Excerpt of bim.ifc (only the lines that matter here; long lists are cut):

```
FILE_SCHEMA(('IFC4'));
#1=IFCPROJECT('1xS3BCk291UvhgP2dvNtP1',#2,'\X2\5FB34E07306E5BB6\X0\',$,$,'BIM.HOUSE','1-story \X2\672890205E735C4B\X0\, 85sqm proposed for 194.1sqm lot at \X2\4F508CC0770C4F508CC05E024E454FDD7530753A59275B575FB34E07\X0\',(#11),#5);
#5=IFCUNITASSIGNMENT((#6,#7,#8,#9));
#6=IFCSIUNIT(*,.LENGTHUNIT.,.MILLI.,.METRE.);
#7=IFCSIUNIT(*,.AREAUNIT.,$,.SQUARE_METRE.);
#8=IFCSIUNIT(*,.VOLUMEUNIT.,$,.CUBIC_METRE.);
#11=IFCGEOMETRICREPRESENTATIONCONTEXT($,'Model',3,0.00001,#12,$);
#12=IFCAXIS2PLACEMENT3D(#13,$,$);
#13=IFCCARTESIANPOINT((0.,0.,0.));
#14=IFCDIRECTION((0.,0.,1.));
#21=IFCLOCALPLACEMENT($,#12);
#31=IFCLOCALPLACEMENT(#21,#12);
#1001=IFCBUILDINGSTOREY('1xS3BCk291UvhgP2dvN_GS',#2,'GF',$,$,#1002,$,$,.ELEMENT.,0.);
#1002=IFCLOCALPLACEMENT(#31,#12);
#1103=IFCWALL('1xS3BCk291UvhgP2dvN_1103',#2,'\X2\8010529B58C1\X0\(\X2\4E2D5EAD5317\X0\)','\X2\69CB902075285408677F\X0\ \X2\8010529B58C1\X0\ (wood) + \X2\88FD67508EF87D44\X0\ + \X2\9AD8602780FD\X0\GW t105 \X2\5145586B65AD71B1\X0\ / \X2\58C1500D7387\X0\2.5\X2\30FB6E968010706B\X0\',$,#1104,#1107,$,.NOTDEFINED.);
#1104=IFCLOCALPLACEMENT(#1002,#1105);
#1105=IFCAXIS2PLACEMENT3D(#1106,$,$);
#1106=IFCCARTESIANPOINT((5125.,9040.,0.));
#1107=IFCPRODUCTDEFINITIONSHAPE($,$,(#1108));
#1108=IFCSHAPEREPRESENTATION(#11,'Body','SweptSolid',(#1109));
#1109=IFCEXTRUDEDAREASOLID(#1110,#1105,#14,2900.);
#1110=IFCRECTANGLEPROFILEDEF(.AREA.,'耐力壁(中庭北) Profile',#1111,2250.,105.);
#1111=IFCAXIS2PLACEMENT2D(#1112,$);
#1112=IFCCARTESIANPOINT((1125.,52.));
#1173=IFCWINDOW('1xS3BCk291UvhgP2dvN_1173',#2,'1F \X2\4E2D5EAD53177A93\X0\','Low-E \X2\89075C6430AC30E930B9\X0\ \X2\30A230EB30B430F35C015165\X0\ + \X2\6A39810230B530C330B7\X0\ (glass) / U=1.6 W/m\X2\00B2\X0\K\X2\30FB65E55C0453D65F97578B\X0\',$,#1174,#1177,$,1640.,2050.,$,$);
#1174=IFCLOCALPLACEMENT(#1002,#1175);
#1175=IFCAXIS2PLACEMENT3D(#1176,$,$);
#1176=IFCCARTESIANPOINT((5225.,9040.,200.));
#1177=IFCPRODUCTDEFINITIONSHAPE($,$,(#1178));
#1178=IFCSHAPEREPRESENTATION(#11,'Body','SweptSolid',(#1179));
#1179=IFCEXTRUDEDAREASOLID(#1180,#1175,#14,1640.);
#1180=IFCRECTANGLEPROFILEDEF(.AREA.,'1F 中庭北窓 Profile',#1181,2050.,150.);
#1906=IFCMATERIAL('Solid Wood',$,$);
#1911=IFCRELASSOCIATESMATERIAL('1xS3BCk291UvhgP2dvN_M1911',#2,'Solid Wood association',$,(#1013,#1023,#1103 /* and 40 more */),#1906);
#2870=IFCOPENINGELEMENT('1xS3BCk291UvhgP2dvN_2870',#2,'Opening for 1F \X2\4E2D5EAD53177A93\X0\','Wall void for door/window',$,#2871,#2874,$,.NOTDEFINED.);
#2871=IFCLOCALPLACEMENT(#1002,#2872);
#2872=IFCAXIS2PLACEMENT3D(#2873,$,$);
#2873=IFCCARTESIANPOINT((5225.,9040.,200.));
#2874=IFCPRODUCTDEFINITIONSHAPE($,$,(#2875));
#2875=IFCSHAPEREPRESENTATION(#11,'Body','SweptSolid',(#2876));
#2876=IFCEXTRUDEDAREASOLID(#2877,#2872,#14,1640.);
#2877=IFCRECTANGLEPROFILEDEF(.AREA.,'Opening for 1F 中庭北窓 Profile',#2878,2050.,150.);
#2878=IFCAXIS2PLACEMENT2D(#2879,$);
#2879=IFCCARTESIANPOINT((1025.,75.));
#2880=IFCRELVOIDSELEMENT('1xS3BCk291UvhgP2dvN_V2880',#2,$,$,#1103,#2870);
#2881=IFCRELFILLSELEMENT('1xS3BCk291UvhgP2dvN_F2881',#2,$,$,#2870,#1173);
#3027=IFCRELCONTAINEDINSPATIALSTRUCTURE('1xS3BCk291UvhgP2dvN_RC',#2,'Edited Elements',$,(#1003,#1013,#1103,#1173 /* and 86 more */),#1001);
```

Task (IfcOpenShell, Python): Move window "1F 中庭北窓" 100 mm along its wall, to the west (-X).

```python
import ifcopenshell
import ifcopenshell.api.geometry
import ifcopenshell.util.placement
import ifcopenshell.util.unit

model = ifcopenshell.open("bim.ifc")
unit_scale = ifcopenshell.util.unit.calculate_unit_scale(model)

window = model.by_id(1173)
opening = window.FillsVoids[0].RelatingOpeningElement
wall = opening.VoidsElements[0].RelatingBuildingElement

wall_matrix = ifcopenshell.util.placement.get_local_placement(wall.ObjectPlacement)
shift = wall_matrix[:3, 0] * -0.1 / unit_scale
before = ifcopenshell.util.placement.get_local_placement(window.ObjectPlacement)[:3, 3].copy()

# The window is not placed relative to its opening, so move both.
for product in (opening, window):
    matrix = ifcopenshell.util.placement.get_local_placement(product.ObjectPlacement)
    matrix[:3, 3] += shift
    ifcopenshell.api.geometry.edit_object_placement(model, product=product, matrix=matrix, is_si=False)

after = ifcopenshell.util.placement.get_local_placement(window.ObjectPlacement)[:3, 3]
print("window moved by", (after - before).round(3) + 0.0)

model.write("bim_v2.ifc")
```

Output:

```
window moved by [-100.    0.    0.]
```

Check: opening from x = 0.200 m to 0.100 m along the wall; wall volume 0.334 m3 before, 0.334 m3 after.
